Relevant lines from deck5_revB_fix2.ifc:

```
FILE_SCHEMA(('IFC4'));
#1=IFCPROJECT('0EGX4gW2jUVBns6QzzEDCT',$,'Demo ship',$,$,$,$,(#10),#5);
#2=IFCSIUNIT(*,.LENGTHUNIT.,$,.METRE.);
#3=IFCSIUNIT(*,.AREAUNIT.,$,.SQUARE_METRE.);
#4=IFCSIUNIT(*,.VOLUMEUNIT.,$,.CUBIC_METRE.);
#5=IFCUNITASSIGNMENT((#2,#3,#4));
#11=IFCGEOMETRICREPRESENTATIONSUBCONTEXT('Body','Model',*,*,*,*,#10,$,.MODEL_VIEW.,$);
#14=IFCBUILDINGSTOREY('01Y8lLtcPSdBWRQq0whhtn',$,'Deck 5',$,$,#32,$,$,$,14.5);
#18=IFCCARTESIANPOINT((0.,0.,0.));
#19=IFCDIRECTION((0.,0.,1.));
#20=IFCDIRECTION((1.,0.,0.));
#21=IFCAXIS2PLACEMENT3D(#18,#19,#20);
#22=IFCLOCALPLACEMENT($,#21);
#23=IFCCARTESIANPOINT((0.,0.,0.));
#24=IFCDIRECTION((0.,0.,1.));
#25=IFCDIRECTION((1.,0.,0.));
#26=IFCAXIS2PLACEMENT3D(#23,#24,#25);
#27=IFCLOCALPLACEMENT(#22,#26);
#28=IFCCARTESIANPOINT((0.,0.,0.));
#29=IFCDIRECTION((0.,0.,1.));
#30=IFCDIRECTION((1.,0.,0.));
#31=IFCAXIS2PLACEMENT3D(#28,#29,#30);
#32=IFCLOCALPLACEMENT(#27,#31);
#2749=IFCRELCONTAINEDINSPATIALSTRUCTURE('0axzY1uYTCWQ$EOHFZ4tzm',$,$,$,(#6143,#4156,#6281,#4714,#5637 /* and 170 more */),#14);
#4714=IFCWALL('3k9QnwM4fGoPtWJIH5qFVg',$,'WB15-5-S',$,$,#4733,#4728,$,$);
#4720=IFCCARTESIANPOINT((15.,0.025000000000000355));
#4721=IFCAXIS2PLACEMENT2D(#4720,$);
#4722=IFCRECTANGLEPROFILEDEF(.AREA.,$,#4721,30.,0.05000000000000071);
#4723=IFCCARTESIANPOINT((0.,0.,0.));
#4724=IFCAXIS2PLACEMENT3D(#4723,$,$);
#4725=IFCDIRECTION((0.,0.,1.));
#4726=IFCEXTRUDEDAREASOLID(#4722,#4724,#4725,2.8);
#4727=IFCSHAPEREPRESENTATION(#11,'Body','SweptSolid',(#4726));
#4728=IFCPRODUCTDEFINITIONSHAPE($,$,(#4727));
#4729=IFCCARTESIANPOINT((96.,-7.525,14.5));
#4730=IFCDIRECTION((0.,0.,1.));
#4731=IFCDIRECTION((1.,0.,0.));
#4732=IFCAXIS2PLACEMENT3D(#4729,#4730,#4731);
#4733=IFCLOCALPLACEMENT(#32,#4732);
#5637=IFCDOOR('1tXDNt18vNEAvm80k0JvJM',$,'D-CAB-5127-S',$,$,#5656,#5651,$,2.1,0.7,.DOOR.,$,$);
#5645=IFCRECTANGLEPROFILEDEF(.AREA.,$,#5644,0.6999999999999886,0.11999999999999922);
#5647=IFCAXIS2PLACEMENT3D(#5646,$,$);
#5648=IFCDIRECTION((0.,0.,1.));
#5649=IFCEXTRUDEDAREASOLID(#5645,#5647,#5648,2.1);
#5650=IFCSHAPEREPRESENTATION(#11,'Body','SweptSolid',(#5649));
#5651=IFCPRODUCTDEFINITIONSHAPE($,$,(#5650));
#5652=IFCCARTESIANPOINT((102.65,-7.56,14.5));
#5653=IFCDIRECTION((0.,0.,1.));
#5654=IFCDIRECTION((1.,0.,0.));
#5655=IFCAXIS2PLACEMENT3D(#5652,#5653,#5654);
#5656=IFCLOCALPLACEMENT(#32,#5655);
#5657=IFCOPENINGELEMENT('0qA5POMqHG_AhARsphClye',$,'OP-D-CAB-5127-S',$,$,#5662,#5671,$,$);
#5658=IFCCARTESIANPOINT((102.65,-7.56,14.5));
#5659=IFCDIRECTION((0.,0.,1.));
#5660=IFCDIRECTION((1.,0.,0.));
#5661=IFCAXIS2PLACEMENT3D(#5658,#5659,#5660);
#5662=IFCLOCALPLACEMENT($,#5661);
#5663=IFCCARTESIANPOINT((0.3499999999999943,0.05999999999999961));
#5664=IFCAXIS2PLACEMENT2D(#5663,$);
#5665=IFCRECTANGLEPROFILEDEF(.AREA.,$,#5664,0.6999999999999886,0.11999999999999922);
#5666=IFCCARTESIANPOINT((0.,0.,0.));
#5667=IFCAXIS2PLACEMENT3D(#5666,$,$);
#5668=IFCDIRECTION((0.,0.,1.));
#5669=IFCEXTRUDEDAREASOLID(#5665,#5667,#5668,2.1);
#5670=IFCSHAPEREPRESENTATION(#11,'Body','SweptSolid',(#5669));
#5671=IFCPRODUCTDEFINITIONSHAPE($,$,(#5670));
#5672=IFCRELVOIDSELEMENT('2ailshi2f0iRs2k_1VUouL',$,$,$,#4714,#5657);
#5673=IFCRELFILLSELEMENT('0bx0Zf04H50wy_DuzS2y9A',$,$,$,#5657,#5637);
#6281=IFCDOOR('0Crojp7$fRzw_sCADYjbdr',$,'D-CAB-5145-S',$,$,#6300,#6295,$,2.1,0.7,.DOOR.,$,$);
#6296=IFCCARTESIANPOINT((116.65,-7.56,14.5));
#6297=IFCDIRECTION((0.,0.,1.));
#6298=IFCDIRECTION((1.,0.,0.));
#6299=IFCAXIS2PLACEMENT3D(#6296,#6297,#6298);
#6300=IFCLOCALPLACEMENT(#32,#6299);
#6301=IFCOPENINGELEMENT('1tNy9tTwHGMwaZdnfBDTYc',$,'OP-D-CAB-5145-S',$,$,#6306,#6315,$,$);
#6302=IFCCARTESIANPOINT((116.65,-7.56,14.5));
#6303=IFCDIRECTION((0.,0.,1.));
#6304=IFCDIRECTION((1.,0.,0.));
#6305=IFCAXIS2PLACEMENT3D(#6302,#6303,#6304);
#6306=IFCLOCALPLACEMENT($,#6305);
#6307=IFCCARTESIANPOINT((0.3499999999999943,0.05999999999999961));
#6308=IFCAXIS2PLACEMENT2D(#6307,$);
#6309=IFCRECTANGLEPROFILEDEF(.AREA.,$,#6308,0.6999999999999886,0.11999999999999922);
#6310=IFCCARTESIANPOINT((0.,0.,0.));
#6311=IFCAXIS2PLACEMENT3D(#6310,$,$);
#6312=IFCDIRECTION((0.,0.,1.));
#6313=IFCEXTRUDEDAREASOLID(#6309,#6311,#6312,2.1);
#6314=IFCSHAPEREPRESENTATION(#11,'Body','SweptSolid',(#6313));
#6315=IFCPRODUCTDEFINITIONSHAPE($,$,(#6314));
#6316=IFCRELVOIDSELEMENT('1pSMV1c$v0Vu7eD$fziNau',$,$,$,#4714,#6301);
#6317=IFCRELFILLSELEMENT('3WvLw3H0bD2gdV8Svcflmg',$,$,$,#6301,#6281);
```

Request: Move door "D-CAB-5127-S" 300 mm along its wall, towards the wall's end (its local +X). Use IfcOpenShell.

```python
import ifcopenshell
import ifcopenshell.api.geometry
import ifcopenshell.util.placement
import ifcopenshell.util.unit

model = ifcopenshell.open("deck5_revB_fix2.ifc")
unit_scale = ifcopenshell.util.unit.calculate_unit_scale(model)

door = model.by_id(5637)
opening = door.FillsVoids[0].RelatingOpeningElement
wall = opening.VoidsElements[0].RelatingBuildingElement

wall_matrix = ifcopenshell.util.placement.get_local_placement(wall.ObjectPlacement)
shift = wall_matrix[:3, 0] * 0.3 / unit_scale
before = ifcopenshell.util.placement.get_local_placement(door.ObjectPlacement)[:3, 3].copy()

# The door is not placed relative to its opening, so move both.
for product in (opening, door):
    matrix = ifcopenshell.util.placement.get_local_placement(product.ObjectPlacement)
    matrix[:3, 3] += shift
    ifcopenshell.api.geometry.edit_object_placement(model, product=product, matrix=matrix, is_si=False)

after = ifcopenshell.util.placement.get_local_placement(door.ObjectPlacement)[:3, 3]
print("door moved by", (after - before).round(3) + 0.0)

model.write("deck5_revB_fix2-out.ifc")
```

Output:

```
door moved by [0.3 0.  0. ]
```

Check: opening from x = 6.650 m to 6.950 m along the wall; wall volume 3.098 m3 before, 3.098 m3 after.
